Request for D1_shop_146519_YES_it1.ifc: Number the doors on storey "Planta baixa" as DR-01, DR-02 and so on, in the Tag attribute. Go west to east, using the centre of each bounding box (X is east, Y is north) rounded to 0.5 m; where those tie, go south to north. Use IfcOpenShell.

First a look at what the model holds.

```python
import ifcopenshell
import ifcopenshell.util.element
import ifcopenshell.util.placement

model = ifcopenshell.open("D1_shop_146519_YES_it1.ifc")
print(model.schema)
storey = next(s for s in model.by_type("IfcBuildingStorey") if s.Name == "Planta baixa")
doors = [e for e in ifcopenshell.util.element.get_decomposition(storey) if e.is_a("IfcDoor")]
for e in sorted(doors, key=lambda e: e.id()):
    origin = ifcopenshell.util.placement.get_local_placement(e.ObjectPlacement)[:3, 3]
    print(e.id(), e.Tag, e.Name, origin.round(2) + 0.0, sep=" | ")
```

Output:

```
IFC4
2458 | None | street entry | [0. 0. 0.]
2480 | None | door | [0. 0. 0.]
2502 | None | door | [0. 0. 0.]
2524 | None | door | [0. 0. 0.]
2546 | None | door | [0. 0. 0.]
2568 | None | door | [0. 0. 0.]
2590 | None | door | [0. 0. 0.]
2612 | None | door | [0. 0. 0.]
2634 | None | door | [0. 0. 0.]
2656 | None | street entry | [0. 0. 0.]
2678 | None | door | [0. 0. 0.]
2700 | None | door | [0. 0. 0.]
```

```python
import ifcopenshell
import ifcopenshell.geom
import ifcopenshell.util.element
import ifcopenshell.util.shape

model = ifcopenshell.open("D1_shop_146519_YES_it1.ifc")
settings = ifcopenshell.geom.settings()
settings.set("use-world-coords", True)


def centre(element):
    shape = ifcopenshell.geom.create_shape(settings, element)
    return ifcopenshell.util.shape.get_bbox_centroid(shape.geometry)


storey = next(s for s in model.by_type("IfcBuildingStorey") if s.Name == "Planta baixa")
doors = [e for e in ifcopenshell.util.element.get_decomposition(storey) if e.is_a("IfcDoor")]

# Insertion points can sit at a corner or the storey origin, so sort by the geometry (in metres).
centres = {e: centre(e) for e in doors}
doors.sort(key=lambda e: (round(centres[e][0] / 0.5), centres[e][1]))

for i, e in enumerate(doors, start=1):
    number = f"DR-{i:02d}"
    e.Tag = number
    print(e.id(), number)

model.write("D1_shop_146519_YES_it1_v2.ifc")
```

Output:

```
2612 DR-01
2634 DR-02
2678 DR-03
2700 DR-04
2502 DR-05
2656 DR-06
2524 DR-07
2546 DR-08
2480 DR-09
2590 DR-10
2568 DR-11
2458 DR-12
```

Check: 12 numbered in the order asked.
